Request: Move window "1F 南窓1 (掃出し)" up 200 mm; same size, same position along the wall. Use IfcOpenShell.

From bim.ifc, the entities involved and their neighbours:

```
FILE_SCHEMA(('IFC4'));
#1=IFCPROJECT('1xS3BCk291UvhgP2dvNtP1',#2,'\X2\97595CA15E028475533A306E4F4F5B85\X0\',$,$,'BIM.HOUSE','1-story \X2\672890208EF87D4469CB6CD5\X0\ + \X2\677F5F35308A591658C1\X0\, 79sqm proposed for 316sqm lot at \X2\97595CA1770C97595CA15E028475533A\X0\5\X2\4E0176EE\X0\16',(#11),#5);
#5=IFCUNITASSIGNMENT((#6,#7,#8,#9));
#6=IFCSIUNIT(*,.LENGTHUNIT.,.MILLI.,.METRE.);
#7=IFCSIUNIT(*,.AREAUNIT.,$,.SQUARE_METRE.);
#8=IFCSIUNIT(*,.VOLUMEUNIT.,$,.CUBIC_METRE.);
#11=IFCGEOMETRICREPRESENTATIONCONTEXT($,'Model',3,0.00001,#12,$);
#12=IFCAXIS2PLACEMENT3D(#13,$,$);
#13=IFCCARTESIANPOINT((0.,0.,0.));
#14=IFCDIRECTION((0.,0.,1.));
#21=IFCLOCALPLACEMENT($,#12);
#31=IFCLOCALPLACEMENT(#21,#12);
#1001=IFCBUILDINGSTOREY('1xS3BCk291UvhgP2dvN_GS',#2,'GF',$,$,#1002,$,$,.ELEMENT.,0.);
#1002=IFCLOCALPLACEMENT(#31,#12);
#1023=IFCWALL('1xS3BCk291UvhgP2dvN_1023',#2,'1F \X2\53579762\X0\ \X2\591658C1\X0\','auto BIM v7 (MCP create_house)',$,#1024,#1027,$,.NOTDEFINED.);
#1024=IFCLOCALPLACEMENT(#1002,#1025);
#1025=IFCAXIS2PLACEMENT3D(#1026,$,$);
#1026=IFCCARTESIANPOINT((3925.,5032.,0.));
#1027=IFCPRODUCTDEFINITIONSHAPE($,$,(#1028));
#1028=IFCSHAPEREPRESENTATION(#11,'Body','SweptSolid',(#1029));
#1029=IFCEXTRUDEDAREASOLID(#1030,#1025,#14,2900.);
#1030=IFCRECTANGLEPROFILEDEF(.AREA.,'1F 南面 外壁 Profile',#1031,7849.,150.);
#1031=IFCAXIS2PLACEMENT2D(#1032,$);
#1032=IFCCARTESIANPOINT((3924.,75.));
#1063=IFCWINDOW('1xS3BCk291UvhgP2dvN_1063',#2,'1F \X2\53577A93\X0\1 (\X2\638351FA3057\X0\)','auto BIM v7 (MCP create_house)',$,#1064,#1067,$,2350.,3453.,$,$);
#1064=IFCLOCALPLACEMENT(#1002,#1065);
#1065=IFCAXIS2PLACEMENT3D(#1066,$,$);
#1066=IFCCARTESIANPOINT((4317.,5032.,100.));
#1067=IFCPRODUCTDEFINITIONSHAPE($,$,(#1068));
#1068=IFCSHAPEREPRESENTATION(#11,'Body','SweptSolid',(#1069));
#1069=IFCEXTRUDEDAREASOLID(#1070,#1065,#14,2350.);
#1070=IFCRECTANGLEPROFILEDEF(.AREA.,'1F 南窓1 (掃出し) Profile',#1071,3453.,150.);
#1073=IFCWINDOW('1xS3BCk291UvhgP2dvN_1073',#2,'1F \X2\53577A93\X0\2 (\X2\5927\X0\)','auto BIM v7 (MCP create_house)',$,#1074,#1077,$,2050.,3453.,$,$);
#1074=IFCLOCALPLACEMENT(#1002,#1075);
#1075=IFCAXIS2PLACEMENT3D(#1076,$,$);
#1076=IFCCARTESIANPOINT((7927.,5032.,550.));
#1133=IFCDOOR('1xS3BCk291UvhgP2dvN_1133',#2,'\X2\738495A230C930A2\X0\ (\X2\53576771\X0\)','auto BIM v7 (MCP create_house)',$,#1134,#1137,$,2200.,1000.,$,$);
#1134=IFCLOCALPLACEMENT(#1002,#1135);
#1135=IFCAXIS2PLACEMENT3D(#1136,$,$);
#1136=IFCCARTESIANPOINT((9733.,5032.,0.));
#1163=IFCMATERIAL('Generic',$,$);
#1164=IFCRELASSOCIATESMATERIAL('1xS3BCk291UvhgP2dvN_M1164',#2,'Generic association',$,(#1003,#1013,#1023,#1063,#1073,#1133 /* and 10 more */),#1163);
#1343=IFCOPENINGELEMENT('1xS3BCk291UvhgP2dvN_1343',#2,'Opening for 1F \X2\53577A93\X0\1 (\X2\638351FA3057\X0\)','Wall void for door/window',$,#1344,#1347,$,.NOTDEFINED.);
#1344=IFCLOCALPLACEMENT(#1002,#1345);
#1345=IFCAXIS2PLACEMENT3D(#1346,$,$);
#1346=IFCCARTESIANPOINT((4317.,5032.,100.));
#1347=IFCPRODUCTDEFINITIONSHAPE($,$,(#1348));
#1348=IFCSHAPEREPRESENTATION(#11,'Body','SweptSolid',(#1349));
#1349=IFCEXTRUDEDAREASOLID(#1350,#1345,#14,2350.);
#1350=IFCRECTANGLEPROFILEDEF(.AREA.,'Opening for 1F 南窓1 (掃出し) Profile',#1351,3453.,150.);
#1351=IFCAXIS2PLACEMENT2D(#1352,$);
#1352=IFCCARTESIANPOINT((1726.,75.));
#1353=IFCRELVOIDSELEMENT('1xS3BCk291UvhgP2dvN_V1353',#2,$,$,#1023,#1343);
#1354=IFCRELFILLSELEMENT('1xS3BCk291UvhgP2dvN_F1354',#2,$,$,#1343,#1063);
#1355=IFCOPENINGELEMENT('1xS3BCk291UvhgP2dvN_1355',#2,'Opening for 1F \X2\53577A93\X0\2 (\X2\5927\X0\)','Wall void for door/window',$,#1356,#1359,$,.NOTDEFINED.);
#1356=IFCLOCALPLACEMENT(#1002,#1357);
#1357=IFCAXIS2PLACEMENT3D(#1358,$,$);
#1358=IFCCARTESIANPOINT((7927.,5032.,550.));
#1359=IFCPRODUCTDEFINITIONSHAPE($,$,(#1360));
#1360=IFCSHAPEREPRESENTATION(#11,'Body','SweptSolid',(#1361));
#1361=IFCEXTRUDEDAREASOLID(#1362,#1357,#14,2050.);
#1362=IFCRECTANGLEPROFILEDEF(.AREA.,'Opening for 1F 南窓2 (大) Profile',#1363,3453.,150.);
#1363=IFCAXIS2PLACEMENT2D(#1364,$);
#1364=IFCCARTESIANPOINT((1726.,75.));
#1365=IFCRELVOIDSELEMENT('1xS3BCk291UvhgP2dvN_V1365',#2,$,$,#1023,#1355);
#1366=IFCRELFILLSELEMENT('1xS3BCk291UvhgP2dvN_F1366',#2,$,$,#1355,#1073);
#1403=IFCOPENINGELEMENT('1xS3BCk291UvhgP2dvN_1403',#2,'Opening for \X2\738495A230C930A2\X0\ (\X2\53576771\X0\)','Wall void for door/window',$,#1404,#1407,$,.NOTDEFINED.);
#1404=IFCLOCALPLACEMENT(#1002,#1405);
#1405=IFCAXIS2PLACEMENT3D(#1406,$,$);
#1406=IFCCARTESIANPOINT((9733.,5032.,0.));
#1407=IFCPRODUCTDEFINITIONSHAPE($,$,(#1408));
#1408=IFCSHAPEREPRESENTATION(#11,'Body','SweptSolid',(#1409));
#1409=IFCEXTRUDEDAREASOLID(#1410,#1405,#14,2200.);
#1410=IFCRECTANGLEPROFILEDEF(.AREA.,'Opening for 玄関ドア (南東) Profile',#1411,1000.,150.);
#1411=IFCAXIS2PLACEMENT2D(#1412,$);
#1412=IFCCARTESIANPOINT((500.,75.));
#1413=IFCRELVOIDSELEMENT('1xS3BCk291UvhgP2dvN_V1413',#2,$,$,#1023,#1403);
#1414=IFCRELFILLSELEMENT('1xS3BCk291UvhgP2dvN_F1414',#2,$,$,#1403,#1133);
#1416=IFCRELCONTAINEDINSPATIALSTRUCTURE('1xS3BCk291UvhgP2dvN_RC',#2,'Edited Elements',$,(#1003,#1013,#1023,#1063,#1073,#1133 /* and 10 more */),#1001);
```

```python
import numpy as np
import ifcopenshell
import ifcopenshell.api.geometry
import ifcopenshell.util.placement
import ifcopenshell.util.unit

model = ifcopenshell.open("bim.ifc")
unit_scale = ifcopenshell.util.unit.calculate_unit_scale(model)

window = model.by_id(1063)
opening = window.FillsVoids[0].RelatingOpeningElement
dz = 0.2 / unit_scale

shift = np.array([0.0, 0.0, dz])
# The window is not placed relative to its opening, so move both.
for product in (opening, window):
    matrix = ifcopenshell.util.placement.get_local_placement(product.ObjectPlacement)
    matrix[:3, 3] += shift
    ifcopenshell.api.geometry.edit_object_placement(model, product=product, matrix=matrix, is_si=False)

print(f"moved by {dz * unit_scale:+.3f} m")

model.write("bim-out.ifc")
```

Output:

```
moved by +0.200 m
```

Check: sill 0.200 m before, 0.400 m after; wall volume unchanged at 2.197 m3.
